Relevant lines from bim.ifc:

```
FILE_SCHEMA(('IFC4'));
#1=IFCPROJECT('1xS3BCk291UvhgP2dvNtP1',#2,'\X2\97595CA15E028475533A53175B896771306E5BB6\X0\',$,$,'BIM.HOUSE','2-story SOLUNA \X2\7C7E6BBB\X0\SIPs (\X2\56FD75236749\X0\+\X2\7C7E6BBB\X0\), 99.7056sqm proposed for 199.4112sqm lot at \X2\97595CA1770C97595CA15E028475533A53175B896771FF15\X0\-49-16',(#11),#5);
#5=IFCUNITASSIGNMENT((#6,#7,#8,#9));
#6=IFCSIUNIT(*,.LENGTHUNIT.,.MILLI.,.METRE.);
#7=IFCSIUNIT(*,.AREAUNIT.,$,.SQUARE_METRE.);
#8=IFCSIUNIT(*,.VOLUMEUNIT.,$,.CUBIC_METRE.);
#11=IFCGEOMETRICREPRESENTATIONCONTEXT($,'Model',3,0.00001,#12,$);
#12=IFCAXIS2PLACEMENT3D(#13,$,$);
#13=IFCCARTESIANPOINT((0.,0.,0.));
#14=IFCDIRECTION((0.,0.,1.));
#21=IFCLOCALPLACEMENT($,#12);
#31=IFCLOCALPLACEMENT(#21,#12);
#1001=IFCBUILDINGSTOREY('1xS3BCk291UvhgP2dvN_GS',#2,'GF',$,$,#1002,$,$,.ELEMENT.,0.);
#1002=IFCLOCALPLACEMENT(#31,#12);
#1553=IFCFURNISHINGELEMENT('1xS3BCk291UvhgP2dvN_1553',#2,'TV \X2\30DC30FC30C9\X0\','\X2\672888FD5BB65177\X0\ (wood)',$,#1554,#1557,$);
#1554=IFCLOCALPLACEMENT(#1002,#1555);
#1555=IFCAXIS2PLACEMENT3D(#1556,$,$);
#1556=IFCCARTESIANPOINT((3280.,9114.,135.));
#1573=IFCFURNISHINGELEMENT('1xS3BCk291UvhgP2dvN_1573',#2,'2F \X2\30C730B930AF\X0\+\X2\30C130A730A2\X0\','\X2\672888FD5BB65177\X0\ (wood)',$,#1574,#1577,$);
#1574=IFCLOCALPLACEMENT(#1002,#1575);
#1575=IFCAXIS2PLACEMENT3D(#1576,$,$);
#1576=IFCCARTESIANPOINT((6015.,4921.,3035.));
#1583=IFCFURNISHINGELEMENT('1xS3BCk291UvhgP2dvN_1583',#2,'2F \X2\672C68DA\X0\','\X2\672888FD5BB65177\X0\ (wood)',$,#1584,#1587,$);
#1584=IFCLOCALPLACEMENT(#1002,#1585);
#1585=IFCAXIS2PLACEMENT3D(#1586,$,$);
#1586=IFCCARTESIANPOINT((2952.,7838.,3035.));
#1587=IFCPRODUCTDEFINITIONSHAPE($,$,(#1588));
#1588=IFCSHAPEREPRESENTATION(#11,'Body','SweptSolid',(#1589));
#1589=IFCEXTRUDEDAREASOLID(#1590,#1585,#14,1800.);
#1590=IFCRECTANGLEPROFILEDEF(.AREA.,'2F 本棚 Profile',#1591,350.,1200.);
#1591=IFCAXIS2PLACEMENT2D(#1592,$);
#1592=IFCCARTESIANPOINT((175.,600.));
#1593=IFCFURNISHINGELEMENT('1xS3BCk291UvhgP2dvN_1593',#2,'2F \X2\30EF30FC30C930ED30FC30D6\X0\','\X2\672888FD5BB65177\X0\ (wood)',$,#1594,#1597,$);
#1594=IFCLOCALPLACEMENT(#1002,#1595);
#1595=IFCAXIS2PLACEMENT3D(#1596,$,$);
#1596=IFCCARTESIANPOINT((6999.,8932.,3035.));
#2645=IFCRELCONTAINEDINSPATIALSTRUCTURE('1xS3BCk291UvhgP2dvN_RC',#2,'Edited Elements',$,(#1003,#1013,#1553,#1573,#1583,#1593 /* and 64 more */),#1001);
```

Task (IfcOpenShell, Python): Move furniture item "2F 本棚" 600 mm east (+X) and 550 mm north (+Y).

```python
import ifcopenshell
import ifcopenshell.api.geometry
import ifcopenshell.util.placement
import ifcopenshell.util.unit

model = ifcopenshell.open("bim.ifc")
unit_scale = ifcopenshell.util.unit.calculate_unit_scale(model)

item = model.by_guid("1xS3BCk291UvhgP2dvN_1583")
matrix = ifcopenshell.util.placement.get_local_placement(item.ObjectPlacement)
matrix[0, 3] += 0.6 / unit_scale
matrix[1, 3] += 0.55 / unit_scale
ifcopenshell.api.geometry.edit_object_placement(model, product=item, matrix=matrix, is_si=False)

print(ifcopenshell.util.placement.get_local_placement(item.ObjectPlacement).round(3) + 0.0)

model.write("bim-out.ifc")
```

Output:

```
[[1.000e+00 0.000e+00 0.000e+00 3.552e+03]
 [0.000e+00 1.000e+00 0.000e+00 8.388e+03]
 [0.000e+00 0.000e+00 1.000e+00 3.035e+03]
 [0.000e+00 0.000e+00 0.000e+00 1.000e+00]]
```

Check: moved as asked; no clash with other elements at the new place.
